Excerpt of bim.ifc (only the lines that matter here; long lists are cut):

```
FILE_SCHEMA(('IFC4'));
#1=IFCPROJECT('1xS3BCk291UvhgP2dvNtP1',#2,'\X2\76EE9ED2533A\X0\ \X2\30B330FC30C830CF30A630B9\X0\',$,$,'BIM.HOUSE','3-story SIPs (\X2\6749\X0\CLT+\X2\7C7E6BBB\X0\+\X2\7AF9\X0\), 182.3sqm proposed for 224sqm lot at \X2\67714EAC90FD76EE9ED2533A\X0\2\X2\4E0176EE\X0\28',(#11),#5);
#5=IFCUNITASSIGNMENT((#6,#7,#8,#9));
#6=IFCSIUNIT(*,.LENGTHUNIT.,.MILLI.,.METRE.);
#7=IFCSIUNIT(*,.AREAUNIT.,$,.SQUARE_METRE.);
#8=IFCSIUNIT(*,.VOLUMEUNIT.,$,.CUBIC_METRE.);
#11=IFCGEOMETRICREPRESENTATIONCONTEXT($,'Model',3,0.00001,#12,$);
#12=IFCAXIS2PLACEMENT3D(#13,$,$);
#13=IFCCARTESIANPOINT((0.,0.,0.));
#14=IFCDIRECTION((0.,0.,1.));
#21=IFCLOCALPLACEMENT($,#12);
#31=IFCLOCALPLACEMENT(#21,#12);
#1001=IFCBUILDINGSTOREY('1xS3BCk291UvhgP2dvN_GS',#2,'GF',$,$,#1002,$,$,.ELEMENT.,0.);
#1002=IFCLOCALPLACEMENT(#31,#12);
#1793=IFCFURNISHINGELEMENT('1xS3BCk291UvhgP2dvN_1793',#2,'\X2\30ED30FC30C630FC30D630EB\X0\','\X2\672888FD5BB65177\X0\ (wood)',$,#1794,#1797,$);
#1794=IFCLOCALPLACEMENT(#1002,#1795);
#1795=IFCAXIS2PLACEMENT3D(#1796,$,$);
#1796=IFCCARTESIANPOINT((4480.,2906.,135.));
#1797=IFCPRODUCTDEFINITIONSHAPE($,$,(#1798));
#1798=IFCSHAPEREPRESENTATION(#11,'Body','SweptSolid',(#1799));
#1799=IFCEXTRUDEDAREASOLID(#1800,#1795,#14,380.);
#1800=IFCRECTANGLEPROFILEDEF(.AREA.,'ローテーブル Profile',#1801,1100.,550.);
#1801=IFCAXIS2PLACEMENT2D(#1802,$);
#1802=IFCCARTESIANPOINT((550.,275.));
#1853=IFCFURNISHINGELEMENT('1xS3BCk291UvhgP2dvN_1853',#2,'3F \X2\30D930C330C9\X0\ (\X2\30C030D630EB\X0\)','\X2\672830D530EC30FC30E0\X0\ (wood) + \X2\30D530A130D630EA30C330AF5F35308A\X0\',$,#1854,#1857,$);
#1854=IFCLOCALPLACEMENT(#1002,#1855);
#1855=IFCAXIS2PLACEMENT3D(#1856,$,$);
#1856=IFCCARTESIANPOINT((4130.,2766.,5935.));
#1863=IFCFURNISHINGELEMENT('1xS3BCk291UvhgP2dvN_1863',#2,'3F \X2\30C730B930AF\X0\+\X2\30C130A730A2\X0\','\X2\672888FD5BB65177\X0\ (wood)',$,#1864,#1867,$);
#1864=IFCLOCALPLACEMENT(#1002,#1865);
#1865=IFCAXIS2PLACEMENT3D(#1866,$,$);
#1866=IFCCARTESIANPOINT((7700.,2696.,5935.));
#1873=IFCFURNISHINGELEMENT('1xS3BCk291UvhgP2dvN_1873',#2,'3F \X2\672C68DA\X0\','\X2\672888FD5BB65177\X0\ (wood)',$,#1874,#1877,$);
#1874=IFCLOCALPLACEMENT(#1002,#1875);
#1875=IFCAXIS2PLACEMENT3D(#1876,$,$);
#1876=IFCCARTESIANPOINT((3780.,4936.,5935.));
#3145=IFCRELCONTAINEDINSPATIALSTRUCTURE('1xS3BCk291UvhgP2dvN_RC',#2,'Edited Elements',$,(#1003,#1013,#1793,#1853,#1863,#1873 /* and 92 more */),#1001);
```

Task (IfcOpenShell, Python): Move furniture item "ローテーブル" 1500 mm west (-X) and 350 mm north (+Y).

```python
import ifcopenshell
import ifcopenshell.api.geometry
import ifcopenshell.util.placement
import ifcopenshell.util.unit

model = ifcopenshell.open("bim.ifc")
unit_scale = ifcopenshell.util.unit.calculate_unit_scale(model)

item = model.by_guid("1xS3BCk291UvhgP2dvN_1793")
matrix = ifcopenshell.util.placement.get_local_placement(item.ObjectPlacement)
matrix[0, 3] -= 1.5 / unit_scale
matrix[1, 3] += 0.35 / unit_scale
ifcopenshell.api.geometry.edit_object_placement(model, product=item, matrix=matrix, is_si=False)

print(ifcopenshell.util.placement.get_local_placement(item.ObjectPlacement).round(3) + 0.0)

model.write("bim_edited.ifc")
```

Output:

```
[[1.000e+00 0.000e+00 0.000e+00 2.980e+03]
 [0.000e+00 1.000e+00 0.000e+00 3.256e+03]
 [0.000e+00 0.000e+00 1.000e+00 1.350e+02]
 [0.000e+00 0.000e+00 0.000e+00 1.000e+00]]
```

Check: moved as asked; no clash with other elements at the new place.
